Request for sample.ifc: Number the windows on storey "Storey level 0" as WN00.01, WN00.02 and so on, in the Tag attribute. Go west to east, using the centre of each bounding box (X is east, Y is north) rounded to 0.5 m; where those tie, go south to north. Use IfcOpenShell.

First a look at what the model holds.

```python
import ifcopenshell
import ifcopenshell.util.element
import ifcopenshell.util.placement

model = ifcopenshell.open("sample.ifc")
print(model.schema)
storey = next(s for s in model.by_type("IfcBuildingStorey") if s.Name == "Storey level 0")
windows = [e for e in ifcopenshell.util.element.get_decomposition(storey) if e.is_a("IfcWindow")]
for e in sorted(windows, key=lambda e: e.id()):
    origin = ifcopenshell.util.placement.get_local_placement(e.ObjectPlacement)[:3, 3]
    print(e.id(), e.Tag, e.Name, origin.round(2) + 0.0, sep=" | ")
```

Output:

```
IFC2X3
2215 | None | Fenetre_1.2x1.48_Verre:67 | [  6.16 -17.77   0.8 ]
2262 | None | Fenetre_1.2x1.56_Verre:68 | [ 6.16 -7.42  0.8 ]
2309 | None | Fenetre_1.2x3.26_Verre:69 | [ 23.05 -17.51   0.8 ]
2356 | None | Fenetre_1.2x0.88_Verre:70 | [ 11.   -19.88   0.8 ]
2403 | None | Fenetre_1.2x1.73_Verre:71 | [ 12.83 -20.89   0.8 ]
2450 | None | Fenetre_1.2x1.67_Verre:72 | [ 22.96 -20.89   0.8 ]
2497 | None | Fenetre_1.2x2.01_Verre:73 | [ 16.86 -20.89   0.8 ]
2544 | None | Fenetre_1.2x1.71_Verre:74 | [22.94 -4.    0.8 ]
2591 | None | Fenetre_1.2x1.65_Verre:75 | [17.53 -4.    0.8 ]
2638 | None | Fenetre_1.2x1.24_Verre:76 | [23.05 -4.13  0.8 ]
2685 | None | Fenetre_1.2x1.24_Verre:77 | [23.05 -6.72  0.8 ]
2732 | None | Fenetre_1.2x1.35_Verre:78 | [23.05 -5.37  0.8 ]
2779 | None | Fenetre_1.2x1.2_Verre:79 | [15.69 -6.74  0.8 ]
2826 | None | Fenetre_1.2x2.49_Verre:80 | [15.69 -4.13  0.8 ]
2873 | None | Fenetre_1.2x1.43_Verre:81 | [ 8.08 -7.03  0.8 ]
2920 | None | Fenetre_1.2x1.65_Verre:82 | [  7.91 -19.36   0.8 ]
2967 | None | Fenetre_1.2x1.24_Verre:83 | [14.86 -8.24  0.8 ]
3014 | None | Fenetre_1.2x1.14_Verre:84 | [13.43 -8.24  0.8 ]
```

```python
import ifcopenshell
import ifcopenshell.geom
import ifcopenshell.util.element
import ifcopenshell.util.shape

model = ifcopenshell.open("sample.ifc")
settings = ifcopenshell.geom.settings()
settings.set("use-world-coords", True)


def centre(element):
    shape = ifcopenshell.geom.create_shape(settings, element)
    return ifcopenshell.util.shape.get_bbox_centroid(shape.geometry)


storey = next(s for s in model.by_type("IfcBuildingStorey") if s.Name == "Storey level 0")
windows = [e for e in ifcopenshell.util.element.get_decomposition(storey) if e.is_a("IfcWindow")]

# Insertion points can sit at a corner or the storey origin, so sort by the geometry (in metres).
centres = {e: centre(e) for e in windows}
windows.sort(key=lambda e: (round(centres[e][0] / 0.5), centres[e][1]))

for i, e in enumerate(windows, start=1):
    number = f"WN00.{i:02d}"
    e.Tag = number
    print(e.id(), number)

model.write("sample_v2.ifc")
```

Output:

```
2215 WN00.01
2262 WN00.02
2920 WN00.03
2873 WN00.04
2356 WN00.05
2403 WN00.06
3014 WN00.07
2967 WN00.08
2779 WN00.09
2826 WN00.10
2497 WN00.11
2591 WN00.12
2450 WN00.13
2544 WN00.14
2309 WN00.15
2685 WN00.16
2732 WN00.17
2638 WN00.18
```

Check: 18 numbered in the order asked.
